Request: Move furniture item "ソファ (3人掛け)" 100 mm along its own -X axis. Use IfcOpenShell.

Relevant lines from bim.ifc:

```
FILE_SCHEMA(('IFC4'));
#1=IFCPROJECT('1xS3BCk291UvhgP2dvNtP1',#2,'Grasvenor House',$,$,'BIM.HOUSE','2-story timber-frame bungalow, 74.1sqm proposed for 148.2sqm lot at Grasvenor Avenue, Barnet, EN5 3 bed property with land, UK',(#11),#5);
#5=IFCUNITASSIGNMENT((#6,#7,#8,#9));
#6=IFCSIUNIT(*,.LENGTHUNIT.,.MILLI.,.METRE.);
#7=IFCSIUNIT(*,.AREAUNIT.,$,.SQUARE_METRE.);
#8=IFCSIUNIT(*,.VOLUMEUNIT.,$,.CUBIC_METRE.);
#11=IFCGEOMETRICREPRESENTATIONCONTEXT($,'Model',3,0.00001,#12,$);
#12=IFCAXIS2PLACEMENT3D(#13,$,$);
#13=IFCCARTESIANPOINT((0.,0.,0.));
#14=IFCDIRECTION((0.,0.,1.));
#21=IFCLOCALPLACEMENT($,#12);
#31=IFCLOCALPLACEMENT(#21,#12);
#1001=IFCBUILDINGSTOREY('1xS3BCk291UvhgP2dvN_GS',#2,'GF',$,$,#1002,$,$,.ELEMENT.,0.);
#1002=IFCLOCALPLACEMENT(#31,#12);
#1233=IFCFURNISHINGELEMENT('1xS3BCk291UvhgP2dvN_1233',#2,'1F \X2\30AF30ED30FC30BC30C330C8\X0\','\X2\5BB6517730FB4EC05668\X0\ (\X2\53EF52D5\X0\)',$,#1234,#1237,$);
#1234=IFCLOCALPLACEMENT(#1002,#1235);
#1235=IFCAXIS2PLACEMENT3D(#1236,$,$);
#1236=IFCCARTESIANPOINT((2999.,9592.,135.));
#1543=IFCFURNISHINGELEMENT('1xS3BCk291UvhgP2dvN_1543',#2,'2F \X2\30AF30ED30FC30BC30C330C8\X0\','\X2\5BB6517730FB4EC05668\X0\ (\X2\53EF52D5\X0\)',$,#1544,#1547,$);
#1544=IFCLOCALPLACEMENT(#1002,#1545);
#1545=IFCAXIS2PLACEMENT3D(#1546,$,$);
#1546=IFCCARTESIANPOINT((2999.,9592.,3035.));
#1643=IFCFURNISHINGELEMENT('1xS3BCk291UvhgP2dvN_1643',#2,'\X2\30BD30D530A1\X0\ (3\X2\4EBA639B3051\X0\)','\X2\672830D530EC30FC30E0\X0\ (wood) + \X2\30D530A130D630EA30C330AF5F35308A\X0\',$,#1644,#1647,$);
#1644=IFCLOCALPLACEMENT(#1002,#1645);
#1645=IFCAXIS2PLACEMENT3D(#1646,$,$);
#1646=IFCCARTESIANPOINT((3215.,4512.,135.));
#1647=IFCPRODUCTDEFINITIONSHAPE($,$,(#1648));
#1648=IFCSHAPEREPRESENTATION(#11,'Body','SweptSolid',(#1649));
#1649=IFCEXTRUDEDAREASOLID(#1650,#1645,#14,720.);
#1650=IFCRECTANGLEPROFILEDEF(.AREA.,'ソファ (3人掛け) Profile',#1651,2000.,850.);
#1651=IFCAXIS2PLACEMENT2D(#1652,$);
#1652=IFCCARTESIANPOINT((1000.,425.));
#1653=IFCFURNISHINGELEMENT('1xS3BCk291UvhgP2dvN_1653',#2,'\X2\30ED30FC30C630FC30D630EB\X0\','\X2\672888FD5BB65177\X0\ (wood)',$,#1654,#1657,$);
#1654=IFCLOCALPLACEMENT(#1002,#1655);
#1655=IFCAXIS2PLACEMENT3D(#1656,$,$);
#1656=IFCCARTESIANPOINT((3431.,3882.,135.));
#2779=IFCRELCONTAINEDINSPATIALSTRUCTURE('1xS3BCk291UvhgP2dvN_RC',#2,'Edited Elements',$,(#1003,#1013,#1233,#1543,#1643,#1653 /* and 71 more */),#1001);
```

```python
import ifcopenshell
import ifcopenshell.api.geometry
import ifcopenshell.util.placement
import ifcopenshell.util.unit

model = ifcopenshell.open("bim.ifc")
unit_scale = ifcopenshell.util.unit.calculate_unit_scale(model)

item = model.by_guid("1xS3BCk291UvhgP2dvN_1643")
matrix = ifcopenshell.util.placement.get_local_placement(item.ObjectPlacement)
matrix[:3, 3] -= matrix[:3, 0] * 0.1 / unit_scale
ifcopenshell.api.geometry.edit_object_placement(model, product=item, matrix=matrix, is_si=False)

print(ifcopenshell.util.placement.get_local_placement(item.ObjectPlacement).round(3) + 0.0)

model.write("bim_v2.ifc")
```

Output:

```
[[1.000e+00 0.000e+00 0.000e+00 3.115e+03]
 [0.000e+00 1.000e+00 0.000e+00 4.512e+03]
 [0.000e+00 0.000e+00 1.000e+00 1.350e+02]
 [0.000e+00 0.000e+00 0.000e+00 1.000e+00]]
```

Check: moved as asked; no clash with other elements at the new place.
